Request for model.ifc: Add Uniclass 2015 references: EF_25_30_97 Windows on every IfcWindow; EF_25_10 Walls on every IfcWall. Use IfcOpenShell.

First a look at what the model holds.

```python
import ifcopenshell

model = ifcopenshell.open("model.ifc")
print(model.schema)
print("classifications:", [c.Name for c in model.by_type("IfcClassification")])
for ifc_class in ("IfcDoor", "IfcRoof", "IfcStair", "IfcWall", "IfcWindow"):
    print(ifc_class, len(model.by_type(ifc_class)))
```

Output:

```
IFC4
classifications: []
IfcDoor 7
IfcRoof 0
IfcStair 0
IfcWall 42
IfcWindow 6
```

```python
import ifcopenshell
import ifcopenshell.api.classification

model = ifcopenshell.open("model.ifc")

system = ifcopenshell.api.classification.add_classification(model, classification="Uniclass 2015")

codes = {
    "IfcWindow": ("EF_25_30_97", "Windows"),
    "IfcWall": ("EF_25_10", "Walls"),
}
for ifc_class, (code, name) in codes.items():
    products = model.by_type(ifc_class)
    ifcopenshell.api.classification.add_reference(
        model, products=products, classification=system, identification=code, name=name
    )
    print(code, len(products))

model.write("model_v2.ifc")
```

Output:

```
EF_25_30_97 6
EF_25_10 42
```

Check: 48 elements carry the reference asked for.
